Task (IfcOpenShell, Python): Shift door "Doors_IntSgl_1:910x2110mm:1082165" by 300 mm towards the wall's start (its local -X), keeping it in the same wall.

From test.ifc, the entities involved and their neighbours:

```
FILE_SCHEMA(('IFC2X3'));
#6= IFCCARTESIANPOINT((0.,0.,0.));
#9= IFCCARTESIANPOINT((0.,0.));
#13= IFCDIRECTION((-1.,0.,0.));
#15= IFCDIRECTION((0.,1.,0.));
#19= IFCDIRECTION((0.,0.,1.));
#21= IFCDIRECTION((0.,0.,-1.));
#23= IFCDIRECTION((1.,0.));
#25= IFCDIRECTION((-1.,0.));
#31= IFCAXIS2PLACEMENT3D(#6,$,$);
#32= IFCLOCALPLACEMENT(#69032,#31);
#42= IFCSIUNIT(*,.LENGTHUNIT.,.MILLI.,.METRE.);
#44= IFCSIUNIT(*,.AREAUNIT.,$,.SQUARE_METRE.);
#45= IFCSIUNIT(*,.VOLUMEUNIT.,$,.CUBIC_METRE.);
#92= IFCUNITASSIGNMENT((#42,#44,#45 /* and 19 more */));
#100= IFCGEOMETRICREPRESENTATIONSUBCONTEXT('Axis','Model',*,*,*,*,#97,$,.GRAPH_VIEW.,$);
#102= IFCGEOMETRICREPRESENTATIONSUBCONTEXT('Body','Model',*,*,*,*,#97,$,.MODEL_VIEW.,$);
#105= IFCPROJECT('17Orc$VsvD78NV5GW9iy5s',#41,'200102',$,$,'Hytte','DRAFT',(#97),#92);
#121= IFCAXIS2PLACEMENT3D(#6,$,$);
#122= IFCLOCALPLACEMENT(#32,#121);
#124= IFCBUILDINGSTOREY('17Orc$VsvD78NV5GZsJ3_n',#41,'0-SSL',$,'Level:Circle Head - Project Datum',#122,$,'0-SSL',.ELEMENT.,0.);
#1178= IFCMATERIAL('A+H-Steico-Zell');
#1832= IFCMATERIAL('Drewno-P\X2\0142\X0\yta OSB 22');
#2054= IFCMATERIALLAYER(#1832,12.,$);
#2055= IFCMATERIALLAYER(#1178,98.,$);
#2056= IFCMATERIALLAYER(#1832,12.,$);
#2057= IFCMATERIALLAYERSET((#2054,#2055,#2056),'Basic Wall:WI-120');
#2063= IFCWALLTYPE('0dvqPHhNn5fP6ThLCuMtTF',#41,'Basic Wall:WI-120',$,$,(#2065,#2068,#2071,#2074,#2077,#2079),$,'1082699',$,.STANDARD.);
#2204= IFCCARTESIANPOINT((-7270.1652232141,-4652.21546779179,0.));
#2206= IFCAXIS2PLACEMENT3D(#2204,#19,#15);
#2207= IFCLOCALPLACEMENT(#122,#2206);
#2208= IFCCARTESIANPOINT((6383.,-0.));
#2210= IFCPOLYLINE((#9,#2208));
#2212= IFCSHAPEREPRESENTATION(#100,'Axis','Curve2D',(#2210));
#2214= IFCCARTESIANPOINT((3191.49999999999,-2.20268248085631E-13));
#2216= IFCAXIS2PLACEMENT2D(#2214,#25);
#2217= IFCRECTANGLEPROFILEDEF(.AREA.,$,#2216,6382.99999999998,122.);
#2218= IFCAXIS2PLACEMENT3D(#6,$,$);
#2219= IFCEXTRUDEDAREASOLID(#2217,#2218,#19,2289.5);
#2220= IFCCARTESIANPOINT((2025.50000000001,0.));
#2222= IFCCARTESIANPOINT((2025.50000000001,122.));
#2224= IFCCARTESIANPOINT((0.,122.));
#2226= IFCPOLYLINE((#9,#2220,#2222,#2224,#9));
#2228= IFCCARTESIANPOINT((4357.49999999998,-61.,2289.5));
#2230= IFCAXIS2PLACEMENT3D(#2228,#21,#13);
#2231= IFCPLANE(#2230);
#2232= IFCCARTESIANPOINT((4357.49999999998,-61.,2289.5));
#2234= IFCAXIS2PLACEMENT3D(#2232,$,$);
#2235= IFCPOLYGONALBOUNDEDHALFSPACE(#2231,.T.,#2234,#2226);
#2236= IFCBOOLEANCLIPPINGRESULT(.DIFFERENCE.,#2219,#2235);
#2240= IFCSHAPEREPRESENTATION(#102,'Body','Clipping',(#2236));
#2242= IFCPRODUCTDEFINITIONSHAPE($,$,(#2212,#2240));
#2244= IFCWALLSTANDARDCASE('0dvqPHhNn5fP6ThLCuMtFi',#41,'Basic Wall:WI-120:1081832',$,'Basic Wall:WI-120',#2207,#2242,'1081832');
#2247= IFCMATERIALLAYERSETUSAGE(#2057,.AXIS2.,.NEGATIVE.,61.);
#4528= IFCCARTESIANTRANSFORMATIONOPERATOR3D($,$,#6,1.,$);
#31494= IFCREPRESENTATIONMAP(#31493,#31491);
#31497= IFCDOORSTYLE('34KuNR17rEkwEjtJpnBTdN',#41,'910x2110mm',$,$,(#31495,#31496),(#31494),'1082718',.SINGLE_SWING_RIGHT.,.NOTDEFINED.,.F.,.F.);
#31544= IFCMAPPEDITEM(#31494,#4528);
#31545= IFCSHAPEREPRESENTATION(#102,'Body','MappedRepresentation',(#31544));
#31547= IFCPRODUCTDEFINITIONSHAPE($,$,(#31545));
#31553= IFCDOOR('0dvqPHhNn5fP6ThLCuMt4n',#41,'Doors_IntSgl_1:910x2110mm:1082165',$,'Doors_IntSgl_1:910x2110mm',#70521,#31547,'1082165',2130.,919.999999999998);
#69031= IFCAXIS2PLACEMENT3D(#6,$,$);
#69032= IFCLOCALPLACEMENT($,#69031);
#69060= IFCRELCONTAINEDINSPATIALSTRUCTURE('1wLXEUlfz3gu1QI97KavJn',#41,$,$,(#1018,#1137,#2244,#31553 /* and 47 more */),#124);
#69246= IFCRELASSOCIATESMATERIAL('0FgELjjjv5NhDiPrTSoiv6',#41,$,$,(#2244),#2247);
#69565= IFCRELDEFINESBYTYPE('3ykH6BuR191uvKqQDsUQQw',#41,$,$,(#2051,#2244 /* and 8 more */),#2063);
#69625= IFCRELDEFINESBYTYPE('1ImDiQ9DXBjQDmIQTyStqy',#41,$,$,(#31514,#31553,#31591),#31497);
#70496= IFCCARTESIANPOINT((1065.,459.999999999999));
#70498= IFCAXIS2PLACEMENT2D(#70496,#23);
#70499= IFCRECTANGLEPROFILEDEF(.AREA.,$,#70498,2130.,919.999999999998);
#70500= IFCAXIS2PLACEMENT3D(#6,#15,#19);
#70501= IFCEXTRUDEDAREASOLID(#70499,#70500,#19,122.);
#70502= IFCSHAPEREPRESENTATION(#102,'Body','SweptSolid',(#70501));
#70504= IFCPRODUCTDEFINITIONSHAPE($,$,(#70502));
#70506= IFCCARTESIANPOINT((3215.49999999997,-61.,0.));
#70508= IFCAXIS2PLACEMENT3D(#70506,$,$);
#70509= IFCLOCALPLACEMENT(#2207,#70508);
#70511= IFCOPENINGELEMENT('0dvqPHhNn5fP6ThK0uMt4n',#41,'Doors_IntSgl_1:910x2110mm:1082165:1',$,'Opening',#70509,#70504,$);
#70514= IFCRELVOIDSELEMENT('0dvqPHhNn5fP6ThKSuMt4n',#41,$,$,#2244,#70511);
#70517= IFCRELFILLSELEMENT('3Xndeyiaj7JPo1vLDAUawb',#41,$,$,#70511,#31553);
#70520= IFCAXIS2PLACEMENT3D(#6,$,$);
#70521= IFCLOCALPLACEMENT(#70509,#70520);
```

```python
import ifcopenshell
import ifcopenshell.api.geometry
import ifcopenshell.util.placement
import ifcopenshell.util.unit

model = ifcopenshell.open("test.ifc")
unit_scale = ifcopenshell.util.unit.calculate_unit_scale(model)

door = model.by_guid("0dvqPHhNn5fP6ThLCuMt4n")
opening = door.FillsVoids[0].RelatingOpeningElement
wall = opening.VoidsElements[0].RelatingBuildingElement

wall_matrix = ifcopenshell.util.placement.get_local_placement(wall.ObjectPlacement)
shift = wall_matrix[:3, 0] * -0.3 / unit_scale
before = ifcopenshell.util.placement.get_local_placement(door.ObjectPlacement)[:3, 3].copy()

# The door is placed relative to its opening, so it follows when the opening moves.
matrix = ifcopenshell.util.placement.get_local_placement(opening.ObjectPlacement)
matrix[:3, 3] += shift
ifcopenshell.api.geometry.edit_object_placement(
    model, product=opening, matrix=matrix, is_si=False, should_transform_children=True
)

after = ifcopenshell.util.placement.get_local_placement(door.ObjectPlacement)[:3, 3]
print("door moved by", (after - before).round(3) + 0.0)

model.write("test_v2.ifc")
```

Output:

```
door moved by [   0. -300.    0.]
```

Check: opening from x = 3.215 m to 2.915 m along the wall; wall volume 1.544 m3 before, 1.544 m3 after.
